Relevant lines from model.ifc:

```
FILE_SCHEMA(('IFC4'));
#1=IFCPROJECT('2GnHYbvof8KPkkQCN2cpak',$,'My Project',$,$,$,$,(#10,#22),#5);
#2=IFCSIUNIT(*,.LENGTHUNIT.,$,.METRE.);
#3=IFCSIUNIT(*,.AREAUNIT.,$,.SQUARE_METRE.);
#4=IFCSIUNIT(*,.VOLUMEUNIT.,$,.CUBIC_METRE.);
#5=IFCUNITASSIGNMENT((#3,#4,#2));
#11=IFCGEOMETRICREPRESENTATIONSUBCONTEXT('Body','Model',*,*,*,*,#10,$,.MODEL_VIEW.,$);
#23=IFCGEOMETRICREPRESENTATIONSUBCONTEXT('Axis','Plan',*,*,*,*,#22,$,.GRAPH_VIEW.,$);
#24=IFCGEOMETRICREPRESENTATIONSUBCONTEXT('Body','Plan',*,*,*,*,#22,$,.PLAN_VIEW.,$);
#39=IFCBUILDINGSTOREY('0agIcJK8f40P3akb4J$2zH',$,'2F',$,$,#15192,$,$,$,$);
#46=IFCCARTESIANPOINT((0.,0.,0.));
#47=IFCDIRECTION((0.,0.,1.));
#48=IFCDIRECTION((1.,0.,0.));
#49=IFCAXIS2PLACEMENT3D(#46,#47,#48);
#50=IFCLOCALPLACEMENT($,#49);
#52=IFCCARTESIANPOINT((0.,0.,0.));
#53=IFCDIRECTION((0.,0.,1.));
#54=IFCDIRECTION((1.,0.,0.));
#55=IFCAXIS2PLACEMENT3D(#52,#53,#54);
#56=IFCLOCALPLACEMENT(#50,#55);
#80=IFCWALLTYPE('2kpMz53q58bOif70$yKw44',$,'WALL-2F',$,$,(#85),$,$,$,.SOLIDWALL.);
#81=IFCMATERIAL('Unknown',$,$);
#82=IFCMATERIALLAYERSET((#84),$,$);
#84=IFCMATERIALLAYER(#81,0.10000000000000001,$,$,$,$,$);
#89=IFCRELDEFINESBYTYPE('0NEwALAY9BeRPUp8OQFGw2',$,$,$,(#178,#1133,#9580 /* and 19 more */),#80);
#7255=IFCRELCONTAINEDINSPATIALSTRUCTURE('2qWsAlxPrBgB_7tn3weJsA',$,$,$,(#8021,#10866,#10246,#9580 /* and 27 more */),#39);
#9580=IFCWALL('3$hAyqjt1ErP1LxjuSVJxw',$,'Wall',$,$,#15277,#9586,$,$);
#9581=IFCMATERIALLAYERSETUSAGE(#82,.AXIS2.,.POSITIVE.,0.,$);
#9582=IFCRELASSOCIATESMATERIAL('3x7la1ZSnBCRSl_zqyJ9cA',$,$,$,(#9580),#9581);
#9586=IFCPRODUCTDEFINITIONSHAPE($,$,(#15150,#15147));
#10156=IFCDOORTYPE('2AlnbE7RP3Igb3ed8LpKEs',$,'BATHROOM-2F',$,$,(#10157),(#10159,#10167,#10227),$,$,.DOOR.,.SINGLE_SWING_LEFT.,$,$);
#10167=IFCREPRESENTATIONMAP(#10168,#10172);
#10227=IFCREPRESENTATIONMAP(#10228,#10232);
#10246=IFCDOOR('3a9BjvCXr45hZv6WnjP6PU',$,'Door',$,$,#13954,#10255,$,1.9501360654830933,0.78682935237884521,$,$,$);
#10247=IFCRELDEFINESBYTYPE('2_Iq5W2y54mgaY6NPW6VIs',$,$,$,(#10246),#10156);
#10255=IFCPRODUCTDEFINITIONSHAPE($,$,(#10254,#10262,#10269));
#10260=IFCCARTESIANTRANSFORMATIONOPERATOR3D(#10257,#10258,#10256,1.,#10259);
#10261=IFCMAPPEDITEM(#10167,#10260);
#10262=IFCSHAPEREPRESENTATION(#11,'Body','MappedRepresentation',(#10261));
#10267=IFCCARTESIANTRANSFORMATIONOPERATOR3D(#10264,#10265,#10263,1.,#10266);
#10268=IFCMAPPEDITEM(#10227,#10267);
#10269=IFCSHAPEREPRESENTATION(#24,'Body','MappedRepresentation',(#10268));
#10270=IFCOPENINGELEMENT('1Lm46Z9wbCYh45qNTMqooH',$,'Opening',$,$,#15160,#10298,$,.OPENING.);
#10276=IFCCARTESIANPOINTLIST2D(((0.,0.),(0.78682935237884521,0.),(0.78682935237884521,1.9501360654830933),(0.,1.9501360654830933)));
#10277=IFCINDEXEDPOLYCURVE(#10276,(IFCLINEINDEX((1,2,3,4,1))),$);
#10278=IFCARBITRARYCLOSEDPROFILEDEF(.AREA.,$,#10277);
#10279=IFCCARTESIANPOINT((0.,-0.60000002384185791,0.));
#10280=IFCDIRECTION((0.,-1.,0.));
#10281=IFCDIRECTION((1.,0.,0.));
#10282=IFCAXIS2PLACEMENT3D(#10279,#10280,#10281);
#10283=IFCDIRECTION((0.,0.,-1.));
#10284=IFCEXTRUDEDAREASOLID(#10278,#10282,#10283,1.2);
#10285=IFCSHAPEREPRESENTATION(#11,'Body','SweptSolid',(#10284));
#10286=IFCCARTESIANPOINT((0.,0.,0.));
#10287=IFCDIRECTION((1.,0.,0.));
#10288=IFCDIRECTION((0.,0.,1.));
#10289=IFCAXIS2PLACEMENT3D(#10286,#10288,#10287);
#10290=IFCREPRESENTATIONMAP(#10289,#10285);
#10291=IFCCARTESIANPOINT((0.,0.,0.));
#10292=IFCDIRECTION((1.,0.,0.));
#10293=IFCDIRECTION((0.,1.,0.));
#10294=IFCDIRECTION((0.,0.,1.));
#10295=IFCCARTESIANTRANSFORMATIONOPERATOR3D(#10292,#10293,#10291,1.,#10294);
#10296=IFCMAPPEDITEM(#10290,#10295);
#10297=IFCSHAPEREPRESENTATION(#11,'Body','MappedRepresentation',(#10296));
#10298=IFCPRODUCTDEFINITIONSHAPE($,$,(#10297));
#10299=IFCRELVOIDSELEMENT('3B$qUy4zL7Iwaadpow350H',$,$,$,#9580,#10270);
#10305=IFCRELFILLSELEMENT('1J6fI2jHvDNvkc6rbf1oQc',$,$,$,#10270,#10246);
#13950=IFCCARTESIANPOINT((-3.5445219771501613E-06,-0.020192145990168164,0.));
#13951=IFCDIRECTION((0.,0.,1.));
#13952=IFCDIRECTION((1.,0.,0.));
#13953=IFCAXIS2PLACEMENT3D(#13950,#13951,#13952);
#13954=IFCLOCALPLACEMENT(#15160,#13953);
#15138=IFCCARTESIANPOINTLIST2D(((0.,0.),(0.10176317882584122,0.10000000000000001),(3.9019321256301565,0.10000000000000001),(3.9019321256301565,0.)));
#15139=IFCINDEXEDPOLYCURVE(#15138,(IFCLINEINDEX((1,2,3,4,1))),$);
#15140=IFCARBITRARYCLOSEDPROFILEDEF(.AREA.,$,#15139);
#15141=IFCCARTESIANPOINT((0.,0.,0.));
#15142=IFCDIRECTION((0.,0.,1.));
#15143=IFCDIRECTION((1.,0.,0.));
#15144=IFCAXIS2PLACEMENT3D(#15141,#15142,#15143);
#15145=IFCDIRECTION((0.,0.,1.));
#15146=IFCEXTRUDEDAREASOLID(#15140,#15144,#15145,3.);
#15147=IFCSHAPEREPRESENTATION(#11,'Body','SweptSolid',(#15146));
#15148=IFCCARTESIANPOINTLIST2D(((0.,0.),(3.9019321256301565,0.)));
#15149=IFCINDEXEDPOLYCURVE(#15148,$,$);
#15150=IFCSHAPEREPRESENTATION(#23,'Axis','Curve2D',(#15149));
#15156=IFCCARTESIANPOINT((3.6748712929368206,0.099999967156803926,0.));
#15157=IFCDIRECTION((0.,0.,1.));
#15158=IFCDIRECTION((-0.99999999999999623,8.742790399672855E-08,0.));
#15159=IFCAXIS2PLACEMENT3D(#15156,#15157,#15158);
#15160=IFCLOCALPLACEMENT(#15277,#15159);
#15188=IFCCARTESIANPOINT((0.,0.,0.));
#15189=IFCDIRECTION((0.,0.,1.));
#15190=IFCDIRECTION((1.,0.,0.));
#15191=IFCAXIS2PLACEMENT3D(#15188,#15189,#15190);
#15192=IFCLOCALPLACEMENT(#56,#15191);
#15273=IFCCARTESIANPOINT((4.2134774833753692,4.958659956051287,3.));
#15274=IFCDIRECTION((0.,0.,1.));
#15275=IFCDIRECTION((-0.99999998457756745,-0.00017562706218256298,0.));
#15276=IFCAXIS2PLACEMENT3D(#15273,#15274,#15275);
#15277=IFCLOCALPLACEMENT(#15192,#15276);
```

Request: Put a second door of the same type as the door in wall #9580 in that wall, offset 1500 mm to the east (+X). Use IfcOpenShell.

```python
import ifcopenshell
import ifcopenshell.api.feature
import ifcopenshell.api.geometry
import ifcopenshell.api.root
import ifcopenshell.geom
import ifcopenshell.util.element
import ifcopenshell.util.placement
import ifcopenshell.util.shape
import ifcopenshell.util.unit

model = ifcopenshell.open("model.ifc")
unit_scale = ifcopenshell.util.unit.calculate_unit_scale(model)
settings = ifcopenshell.geom.settings()


def volume(element):
    """Net volume in cubic metres, openings subtracted."""
    shape = ifcopenshell.geom.create_shape(settings, element)
    return ifcopenshell.util.shape.get_volume(shape.geometry)


door = model.by_id(10246)
opening = door.FillsVoids[0].RelatingOpeningElement
wall = opening.VoidsElements[0].RelatingBuildingElement
before = volume(wall)
shift = ifcopenshell.util.placement.get_local_placement(wall.ObjectPlacement)[:3, 0] * -1.5 / unit_scale

# copy_class copies the void relationship, type, container and properties, but no geometry.
new_opening = ifcopenshell.api.root.copy_class(model, product=opening)
new_opening.Representation = ifcopenshell.util.element.copy_deep(
    model, opening.Representation, exclude=["IfcGeometricRepresentationContext", "IfcRepresentationMap"]
)
new_door = ifcopenshell.api.root.copy_class(model, product=door)
new_door.Representation = ifcopenshell.util.element.copy_deep(
    model, door.Representation, exclude=["IfcGeometricRepresentationContext", "IfcRepresentationMap"]
)
ifcopenshell.api.feature.add_filling(model, opening=new_opening, element=new_door)

for old, new in ((opening, new_opening), (door, new_door)):
    matrix = ifcopenshell.util.placement.get_local_placement(old.ObjectPlacement)
    matrix[:3, 3] += shift
    ifcopenshell.api.geometry.edit_object_placement(model, product=new, matrix=matrix, is_si=False)

after = volume(wall)

print(f"wall volume {before:.3f} -> {after:.3f} m3")

model.write("model_v2.ifc")
```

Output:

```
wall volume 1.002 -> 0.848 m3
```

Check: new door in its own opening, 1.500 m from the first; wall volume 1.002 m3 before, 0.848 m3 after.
